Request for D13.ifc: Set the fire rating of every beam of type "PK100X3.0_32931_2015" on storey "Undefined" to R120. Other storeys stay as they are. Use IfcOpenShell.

First a look at what the model holds.

```python
import ifcopenshell
import ifcopenshell.util.element

model = ifcopenshell.open("D13.ifc")
print(model.schema)
storey = next(s for s in model.by_type("IfcBuildingStorey") if s.Name == "Undefined")
beams = [e for e in ifcopenshell.util.element.get_decomposition(storey) if e.is_a("IfcBeam")]
seen = {}
for e in beams:
    element_type = ifcopenshell.util.element.get_type(e)
    key = (element_type.Name if element_type != e and element_type else None, ifcopenshell.util.element.get_pset(e, "Pset_BeamCommon", "FireRating"))
    seen[key] = seen.get(key, 0) + 1
for (name, value), count in sorted(seen.items(), key=str):
    print(count, "x", name, "|", value)
```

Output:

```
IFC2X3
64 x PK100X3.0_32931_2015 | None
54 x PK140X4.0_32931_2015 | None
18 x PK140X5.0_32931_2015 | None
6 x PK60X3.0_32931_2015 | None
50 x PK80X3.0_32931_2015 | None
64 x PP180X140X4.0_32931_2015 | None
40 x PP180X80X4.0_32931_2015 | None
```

```python
import ifcopenshell
import ifcopenshell.api.pset
import ifcopenshell.util.element

model = ifcopenshell.open("D13.ifc")

storey = next(s for s in model.by_type("IfcBuildingStorey") if s.Name == "Undefined")
beams = [e for e in ifcopenshell.util.element.get_decomposition(storey) if e.is_a("IfcBeam")]

count = 0
for e in beams:
    element_type = ifcopenshell.util.element.get_type(e)
    if element_type in (None, e) or element_type.Name != "PK100X3.0_32931_2015":
        continue
    found = ifcopenshell.util.element.get_pset(e, "Pset_BeamCommon", should_inherit=False)
    if found:
        pset = model.by_id(found["id"])
        if len(ifcopenshell.util.element.get_elements_by_pset(pset)) > 1:
            pset = ifcopenshell.api.pset.unshare_pset(model, products=[e], pset=pset)[0]
    else:
        pset = ifcopenshell.api.pset.add_pset(model, product=e, name="Pset_BeamCommon")
    ifcopenshell.api.pset.edit_pset(model, pset=pset, properties={"FireRating": "R120"})
    count += 1

print(count, "beams updated")

model.write("D13-out.ifc")
```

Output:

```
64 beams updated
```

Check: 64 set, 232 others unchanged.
